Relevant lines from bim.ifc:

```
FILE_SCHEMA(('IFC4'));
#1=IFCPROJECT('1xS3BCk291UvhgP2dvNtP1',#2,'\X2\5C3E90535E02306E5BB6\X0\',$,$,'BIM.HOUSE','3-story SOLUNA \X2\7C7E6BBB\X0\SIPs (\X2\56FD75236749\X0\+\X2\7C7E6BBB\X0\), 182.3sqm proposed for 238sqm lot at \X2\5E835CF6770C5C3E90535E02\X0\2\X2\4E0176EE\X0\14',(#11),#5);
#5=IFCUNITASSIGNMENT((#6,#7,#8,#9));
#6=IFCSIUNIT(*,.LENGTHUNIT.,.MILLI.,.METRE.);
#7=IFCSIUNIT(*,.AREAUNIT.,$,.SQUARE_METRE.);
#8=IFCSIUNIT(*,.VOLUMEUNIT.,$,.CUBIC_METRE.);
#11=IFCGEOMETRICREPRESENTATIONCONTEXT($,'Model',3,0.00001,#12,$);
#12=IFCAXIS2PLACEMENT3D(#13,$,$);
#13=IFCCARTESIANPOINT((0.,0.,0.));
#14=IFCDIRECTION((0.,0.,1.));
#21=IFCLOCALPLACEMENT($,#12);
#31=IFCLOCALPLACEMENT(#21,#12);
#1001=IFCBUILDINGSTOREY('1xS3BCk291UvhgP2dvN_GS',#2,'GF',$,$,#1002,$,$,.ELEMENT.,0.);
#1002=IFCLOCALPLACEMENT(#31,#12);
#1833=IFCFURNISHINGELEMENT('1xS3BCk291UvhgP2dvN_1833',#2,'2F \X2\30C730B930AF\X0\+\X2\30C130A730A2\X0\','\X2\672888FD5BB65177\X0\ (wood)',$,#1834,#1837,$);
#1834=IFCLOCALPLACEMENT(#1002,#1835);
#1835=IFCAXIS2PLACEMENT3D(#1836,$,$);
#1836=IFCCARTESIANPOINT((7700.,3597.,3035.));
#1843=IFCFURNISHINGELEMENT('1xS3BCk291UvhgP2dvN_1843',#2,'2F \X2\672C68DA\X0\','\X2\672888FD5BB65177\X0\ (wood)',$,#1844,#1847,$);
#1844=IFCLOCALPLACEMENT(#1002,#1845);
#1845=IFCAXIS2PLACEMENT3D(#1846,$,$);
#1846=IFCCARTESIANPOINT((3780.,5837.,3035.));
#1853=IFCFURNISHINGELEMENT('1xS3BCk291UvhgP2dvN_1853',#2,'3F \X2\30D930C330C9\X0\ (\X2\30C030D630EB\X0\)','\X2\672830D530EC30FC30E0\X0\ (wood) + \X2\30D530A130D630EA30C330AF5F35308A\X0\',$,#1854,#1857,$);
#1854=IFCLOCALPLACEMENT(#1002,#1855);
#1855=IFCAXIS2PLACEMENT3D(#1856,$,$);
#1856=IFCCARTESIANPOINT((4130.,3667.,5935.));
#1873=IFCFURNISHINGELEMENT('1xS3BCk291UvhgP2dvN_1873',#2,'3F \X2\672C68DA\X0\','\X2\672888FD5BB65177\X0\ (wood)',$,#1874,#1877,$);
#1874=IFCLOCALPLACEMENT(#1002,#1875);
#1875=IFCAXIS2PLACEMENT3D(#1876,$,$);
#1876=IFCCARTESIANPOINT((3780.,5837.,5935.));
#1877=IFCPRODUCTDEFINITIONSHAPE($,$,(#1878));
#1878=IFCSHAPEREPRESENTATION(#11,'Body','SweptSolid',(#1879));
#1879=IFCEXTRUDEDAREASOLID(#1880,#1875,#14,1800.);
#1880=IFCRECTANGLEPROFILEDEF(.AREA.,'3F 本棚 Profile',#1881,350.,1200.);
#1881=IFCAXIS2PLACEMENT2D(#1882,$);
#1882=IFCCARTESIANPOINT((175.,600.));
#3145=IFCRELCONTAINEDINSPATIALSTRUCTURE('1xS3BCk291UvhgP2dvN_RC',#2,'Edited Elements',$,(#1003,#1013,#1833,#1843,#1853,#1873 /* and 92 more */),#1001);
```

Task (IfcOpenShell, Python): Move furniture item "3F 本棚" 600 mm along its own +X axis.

```python
import ifcopenshell
import ifcopenshell.api.geometry
import ifcopenshell.util.placement

model = ifcopenshell.open("bim.ifc")

item = model.by_guid("1xS3BCk291UvhgP2dvN_1873")
matrix = ifcopenshell.util.placement.get_local_placement(item.ObjectPlacement)
matrix[:3, 3] += matrix[:3, 0] * 600.0
ifcopenshell.api.geometry.edit_object_placement(model, product=item, matrix=matrix, is_si=False)

print(ifcopenshell.util.placement.get_local_placement(item.ObjectPlacement).round(3) + 0.0)

model.write("bim_edited.ifc")
```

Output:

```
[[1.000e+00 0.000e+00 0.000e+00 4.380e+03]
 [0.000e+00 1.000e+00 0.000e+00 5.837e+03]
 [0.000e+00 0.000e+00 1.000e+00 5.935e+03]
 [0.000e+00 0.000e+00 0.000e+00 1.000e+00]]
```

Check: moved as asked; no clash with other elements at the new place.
